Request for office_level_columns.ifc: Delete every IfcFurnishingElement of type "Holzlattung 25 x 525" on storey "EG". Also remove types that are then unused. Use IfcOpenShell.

First a look at what the model holds.

```python
import ifcopenshell
import ifcopenshell.util.element

model = ifcopenshell.open("office_level_columns.ifc")
print(model.schema)
storey = next(s for s in model.by_type("IfcBuildingStorey") if s.Name == "EG")
furniture = [e for e in ifcopenshell.util.element.get_decomposition(storey) if e.is_a("IfcFurnishingElement")]
seen = {}
for e in furniture:
    element_type = ifcopenshell.util.element.get_type(e)
    name = element_type.Name if element_type not in (None, e) else None
    seen[name] = seen.get(name, 0) + 1
for name, count in sorted(seen.items(), key=str):
    print(count, "x", name)
```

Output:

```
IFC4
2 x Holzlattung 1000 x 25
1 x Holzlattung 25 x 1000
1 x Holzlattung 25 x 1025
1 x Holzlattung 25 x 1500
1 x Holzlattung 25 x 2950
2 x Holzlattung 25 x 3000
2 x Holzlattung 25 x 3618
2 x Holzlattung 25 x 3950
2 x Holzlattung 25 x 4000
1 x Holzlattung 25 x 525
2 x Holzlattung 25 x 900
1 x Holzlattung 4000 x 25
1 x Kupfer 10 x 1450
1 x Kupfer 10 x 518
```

```python
import ifcopenshell
import ifcopenshell.api.root
import ifcopenshell.util.element

model = ifcopenshell.open("office_level_columns.ifc")

storey = next(s for s in model.by_type("IfcBuildingStorey") if s.Name == "EG")
furniture = [e for e in ifcopenshell.util.element.get_decomposition(storey) if e.is_a("IfcFurnishingElement")]
targets = [e for e in furniture if (t := ifcopenshell.util.element.get_type(e)) not in (None, e) and t.Name == "Holzlattung 25 x 525"]
types = {ifcopenshell.util.element.get_type(e) for e in targets} - {None, *targets}

for e in targets:
    ifcopenshell.api.root.remove_product(model, product=e)
print(len(targets), "removed")

unused = [t for t in types if not ifcopenshell.util.element.get_types(t)]
for t in unused:
    ifcopenshell.api.root.remove_product(model, product=t)
print(len(unused), "unused types removed")

model.write("office_level_columns_v2.ifc")
```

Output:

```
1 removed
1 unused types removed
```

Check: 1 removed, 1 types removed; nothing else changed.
